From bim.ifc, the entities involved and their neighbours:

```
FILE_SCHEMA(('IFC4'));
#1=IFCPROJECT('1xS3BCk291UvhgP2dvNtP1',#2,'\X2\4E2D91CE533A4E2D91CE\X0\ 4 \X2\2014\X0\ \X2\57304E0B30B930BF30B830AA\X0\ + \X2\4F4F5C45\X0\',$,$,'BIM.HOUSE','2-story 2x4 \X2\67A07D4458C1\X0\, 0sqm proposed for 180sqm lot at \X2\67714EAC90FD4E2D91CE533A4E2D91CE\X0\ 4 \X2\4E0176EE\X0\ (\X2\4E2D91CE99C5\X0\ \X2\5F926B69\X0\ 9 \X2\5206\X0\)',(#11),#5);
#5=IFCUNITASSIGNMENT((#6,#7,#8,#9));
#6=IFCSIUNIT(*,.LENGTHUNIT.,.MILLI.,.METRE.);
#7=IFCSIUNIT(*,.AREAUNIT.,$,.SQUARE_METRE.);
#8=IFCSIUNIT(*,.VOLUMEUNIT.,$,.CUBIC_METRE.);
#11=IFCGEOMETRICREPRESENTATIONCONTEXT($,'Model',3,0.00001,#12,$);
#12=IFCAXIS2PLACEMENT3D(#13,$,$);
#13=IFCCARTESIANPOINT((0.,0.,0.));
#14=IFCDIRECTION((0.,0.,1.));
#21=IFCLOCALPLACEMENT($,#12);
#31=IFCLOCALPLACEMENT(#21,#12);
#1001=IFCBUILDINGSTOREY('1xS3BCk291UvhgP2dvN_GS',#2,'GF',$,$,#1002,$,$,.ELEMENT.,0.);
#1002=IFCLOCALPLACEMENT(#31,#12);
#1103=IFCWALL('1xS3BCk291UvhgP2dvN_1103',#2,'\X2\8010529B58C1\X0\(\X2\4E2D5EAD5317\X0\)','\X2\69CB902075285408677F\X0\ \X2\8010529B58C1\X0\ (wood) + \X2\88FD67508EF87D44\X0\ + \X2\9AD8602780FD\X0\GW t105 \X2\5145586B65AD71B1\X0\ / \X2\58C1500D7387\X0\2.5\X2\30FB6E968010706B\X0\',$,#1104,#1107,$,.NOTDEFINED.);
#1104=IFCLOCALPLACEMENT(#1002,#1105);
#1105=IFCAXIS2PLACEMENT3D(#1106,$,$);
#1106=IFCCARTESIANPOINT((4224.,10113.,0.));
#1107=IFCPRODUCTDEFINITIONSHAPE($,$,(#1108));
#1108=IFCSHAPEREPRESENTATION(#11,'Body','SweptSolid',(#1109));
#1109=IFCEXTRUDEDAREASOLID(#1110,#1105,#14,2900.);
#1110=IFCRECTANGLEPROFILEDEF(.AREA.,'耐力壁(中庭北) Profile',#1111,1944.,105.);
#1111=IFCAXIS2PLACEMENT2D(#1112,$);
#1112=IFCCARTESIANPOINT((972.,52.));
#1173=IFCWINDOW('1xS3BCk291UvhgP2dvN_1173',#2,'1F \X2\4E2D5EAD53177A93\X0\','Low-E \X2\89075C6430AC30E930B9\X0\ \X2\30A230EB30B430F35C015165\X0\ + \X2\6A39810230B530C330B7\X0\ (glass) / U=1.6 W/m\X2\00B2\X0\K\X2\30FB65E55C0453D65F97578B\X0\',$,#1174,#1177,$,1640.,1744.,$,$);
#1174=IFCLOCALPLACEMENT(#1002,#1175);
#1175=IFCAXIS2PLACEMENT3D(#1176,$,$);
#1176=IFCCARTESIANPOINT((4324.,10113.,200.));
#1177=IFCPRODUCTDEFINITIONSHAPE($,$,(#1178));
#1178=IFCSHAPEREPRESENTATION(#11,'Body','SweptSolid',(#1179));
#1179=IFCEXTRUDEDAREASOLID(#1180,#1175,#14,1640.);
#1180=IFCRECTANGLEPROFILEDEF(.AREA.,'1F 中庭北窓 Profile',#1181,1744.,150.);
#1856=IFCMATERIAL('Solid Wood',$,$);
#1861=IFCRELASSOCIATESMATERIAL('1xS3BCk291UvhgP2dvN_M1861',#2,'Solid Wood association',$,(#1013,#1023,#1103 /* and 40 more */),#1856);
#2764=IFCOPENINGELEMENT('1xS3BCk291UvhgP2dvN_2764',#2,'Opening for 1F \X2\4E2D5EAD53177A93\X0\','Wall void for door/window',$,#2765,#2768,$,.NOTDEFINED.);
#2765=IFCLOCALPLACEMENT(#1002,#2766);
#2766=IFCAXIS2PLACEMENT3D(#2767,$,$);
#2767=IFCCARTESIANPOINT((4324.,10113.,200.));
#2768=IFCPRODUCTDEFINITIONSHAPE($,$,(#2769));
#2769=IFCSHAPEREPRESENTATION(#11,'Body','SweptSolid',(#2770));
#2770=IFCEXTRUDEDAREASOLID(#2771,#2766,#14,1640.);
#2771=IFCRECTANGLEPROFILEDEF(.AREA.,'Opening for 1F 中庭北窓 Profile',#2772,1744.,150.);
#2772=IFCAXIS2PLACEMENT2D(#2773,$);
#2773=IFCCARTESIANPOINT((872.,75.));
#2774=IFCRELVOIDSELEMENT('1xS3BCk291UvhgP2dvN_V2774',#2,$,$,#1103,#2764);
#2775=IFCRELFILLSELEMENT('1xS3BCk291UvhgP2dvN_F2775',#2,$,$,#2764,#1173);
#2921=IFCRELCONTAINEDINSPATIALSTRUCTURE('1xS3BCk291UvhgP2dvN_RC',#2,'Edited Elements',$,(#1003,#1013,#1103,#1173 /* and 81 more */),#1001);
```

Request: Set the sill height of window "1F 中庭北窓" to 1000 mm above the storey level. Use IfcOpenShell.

```python
import numpy as np
import ifcopenshell
import ifcopenshell.api.geometry
import ifcopenshell.geom
import ifcopenshell.util.element
import ifcopenshell.util.placement
import ifcopenshell.util.shape
import ifcopenshell.util.unit

model = ifcopenshell.open("bim.ifc")
unit_scale = ifcopenshell.util.unit.calculate_unit_scale(model)

window = model.by_guid("1xS3BCk291UvhgP2dvN_1173")
opening = window.FillsVoids[0].RelatingOpeningElement
storey = ifcopenshell.util.element.get_container(window, ifc_class="IfcBuildingStorey")
level = ifcopenshell.util.placement.get_local_placement(storey.ObjectPlacement)[2, 3]

# The opening's origin need not be at the sill, so measure its lowest point.
shape = ifcopenshell.geom.create_shape(ifcopenshell.geom.settings(), opening)
bottom = ifcopenshell.util.shape.get_shape_bottom_elevation(shape, shape.geometry) / unit_scale
dz = level + 1 / unit_scale - bottom

shift = np.array([0.0, 0.0, dz])
# The window is not placed relative to its opening, so move both.
for product in (opening, window):
    matrix = ifcopenshell.util.placement.get_local_placement(product.ObjectPlacement)
    matrix[:3, 3] += shift
    ifcopenshell.api.geometry.edit_object_placement(model, product=product, matrix=matrix, is_si=False)

print(f"moved by {dz * unit_scale:+.3f} m")

model.write("bim_v2.ifc")
```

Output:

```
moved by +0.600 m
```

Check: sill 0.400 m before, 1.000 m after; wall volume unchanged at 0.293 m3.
